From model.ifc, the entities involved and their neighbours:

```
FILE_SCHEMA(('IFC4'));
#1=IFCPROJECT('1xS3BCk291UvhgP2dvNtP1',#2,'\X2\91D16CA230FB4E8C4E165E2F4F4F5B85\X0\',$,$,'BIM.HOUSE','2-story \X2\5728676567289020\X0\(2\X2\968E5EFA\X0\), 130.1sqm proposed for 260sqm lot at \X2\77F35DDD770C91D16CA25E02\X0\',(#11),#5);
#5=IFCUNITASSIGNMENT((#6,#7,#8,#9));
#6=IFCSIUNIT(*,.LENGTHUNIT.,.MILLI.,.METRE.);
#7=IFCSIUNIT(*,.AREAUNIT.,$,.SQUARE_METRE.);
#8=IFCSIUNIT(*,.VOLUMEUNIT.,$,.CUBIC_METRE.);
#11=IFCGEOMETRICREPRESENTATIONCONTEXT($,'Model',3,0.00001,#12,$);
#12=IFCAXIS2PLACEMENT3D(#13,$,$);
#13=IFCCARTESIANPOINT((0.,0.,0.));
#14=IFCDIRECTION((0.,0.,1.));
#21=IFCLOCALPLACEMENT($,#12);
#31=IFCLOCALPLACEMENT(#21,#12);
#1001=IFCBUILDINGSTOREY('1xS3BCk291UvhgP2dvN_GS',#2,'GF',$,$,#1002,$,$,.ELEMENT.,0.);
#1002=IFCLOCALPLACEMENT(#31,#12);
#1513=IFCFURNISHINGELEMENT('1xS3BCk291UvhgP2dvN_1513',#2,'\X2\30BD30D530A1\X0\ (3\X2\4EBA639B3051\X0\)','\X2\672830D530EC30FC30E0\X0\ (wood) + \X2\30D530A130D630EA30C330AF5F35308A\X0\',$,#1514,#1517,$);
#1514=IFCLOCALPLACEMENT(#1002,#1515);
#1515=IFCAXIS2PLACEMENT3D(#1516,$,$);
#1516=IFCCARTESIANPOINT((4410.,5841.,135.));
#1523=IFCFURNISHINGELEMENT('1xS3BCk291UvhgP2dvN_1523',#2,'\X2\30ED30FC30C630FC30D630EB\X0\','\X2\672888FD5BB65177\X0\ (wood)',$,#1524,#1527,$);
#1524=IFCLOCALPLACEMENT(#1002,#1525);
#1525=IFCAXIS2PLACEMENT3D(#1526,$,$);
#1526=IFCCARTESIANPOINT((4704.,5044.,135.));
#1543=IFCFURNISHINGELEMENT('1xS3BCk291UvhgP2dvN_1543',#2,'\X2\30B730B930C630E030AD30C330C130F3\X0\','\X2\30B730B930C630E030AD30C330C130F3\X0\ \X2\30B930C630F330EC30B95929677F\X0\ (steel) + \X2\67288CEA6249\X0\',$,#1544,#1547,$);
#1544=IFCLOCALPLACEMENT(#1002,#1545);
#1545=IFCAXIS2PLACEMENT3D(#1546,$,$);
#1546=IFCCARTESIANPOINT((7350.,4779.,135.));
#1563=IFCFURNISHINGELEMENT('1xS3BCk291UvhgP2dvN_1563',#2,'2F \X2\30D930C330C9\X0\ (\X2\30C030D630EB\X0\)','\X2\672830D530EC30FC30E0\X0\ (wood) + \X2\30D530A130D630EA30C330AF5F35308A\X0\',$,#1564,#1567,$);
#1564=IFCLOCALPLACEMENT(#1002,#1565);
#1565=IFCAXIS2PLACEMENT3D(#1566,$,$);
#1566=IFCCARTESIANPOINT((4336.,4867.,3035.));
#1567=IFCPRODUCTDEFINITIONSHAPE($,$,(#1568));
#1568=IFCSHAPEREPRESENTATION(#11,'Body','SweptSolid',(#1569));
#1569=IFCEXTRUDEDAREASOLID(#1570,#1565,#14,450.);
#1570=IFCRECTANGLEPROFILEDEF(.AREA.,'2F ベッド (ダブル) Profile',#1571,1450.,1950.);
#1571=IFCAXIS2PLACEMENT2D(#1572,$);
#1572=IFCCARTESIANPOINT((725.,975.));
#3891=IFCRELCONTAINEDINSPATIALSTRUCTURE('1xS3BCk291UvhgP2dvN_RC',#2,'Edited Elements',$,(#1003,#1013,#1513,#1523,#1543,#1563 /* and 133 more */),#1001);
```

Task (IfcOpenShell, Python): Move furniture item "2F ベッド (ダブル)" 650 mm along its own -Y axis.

```python
import ifcopenshell
import ifcopenshell.api.geometry
import ifcopenshell.util.placement
import ifcopenshell.util.unit

model = ifcopenshell.open("model.ifc")
unit_scale = ifcopenshell.util.unit.calculate_unit_scale(model)

item = model.by_guid("1xS3BCk291UvhgP2dvN_1563")
matrix = ifcopenshell.util.placement.get_local_placement(item.ObjectPlacement)
matrix[:3, 3] -= matrix[:3, 1] * 0.65 / unit_scale
ifcopenshell.api.geometry.edit_object_placement(model, product=item, matrix=matrix, is_si=False)

print(ifcopenshell.util.placement.get_local_placement(item.ObjectPlacement).round(3) + 0.0)

model.write("model_v2.ifc")
```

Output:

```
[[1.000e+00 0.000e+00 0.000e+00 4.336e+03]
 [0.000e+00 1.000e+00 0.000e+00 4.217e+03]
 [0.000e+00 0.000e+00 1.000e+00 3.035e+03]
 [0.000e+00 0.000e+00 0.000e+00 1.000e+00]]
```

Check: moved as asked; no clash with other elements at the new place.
